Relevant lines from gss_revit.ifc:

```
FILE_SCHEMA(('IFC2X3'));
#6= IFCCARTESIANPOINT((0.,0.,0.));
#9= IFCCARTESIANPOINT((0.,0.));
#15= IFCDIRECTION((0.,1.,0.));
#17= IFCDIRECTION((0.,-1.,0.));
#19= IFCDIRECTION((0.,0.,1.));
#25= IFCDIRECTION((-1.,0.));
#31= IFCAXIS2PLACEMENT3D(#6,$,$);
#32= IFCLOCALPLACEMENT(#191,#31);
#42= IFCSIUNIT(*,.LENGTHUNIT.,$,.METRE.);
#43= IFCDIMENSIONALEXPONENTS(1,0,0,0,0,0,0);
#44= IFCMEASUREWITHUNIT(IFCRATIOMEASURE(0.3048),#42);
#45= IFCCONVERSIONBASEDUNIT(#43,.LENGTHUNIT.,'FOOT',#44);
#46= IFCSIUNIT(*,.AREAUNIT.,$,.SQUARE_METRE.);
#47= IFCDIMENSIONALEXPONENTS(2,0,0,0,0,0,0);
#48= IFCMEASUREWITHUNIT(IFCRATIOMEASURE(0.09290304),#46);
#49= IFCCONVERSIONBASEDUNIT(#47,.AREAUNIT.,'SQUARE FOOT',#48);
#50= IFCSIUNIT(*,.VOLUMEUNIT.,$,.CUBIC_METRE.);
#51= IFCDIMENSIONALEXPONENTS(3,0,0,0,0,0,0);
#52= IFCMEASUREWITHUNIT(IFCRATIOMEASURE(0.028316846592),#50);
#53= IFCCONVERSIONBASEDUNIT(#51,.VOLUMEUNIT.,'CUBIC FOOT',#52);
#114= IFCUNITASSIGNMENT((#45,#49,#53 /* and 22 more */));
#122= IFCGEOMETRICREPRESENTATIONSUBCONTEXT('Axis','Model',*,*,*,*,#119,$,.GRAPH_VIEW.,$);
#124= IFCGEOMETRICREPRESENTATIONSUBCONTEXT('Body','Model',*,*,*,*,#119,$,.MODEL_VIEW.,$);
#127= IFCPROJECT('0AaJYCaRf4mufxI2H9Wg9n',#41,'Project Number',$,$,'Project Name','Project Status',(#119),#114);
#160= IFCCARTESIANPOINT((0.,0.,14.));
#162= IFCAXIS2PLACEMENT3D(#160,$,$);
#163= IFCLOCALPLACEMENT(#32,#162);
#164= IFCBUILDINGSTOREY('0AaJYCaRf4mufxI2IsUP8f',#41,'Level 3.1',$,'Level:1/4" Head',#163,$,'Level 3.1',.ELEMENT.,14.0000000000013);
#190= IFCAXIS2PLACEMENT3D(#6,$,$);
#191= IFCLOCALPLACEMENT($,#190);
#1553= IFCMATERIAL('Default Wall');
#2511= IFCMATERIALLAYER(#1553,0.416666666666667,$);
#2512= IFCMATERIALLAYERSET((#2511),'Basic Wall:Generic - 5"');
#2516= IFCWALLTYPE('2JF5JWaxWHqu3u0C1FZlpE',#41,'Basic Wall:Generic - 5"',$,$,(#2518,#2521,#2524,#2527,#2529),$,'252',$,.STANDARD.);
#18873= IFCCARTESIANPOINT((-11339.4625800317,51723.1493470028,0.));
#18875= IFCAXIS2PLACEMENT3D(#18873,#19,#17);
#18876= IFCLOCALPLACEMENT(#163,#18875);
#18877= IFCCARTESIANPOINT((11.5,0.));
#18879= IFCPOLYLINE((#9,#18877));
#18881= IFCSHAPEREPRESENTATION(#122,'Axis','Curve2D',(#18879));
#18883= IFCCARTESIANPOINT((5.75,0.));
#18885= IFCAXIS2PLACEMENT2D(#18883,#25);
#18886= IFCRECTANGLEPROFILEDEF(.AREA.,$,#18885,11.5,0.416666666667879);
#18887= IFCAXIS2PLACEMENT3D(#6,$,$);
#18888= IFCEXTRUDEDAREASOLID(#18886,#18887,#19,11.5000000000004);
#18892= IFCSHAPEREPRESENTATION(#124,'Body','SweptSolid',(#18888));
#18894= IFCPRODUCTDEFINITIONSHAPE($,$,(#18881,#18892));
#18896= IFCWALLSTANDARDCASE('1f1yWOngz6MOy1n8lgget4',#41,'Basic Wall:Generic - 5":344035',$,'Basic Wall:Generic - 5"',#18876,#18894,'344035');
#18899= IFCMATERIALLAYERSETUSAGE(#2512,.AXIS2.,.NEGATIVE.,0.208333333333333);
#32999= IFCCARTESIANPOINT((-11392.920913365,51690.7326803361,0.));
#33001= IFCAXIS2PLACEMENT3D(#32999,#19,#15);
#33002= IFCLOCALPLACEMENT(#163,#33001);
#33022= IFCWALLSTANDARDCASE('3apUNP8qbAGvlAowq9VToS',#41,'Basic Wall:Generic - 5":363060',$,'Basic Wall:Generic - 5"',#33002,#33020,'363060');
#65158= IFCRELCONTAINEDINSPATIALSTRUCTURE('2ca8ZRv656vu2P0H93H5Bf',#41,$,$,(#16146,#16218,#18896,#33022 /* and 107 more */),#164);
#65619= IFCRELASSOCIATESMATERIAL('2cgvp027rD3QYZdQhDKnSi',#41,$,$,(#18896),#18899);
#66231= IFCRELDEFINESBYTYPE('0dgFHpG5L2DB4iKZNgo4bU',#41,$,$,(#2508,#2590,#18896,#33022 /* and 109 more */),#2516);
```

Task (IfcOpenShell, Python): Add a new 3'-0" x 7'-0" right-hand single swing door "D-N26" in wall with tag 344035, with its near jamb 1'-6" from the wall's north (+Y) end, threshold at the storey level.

```python
import numpy as np
import ifcopenshell
import ifcopenshell.api.feature
import ifcopenshell.api.geometry
import ifcopenshell.api.root
import ifcopenshell.api.spatial
import ifcopenshell.api.type
import ifcopenshell.geom
import ifcopenshell.util.element
import ifcopenshell.util.placement
import ifcopenshell.util.representation
import ifcopenshell.util.shape
import ifcopenshell.util.unit

model = ifcopenshell.open("gss_revit.ifc")
unit_scale = ifcopenshell.util.unit.calculate_unit_scale(model)
settings = ifcopenshell.geom.settings()


def volume(element):
    """Net volume in cubic metres, openings subtracted."""
    shape = ifcopenshell.geom.create_shape(settings, element)
    return ifcopenshell.util.shape.get_volume(shape.geometry)


wall = model.by_guid("1f1yWOngz6MOy1n8lgget4")
storey = ifcopenshell.util.element.get_container(wall, ifc_class="IfcBuildingStorey")
context = ifcopenshell.util.representation.get_context(model, "Model", "Body", "MODEL_VIEW")
before = volume(wall)

width, height, from_end, sill = 0.9144, 2.1336, 0.4572, 0.0  # metres

# The wall runs along its own X axis, and the end named is its -X end.
wall_shape = ifcopenshell.geom.create_shape(settings, wall)
x, y, z = ifcopenshell.util.shape.get_vertices(wall_shape.geometry).T
start = x.min() + from_end
face, thickness = float(y.min()), float(y.max() - y.min())
wall_matrix = ifcopenshell.util.placement.get_local_placement(wall.ObjectPlacement)
level = ifcopenshell.util.placement.get_local_placement(storey.ObjectPlacement)[2, 3]


def in_wall(x, y):
    """Placement at x, y metres in the wall's axes, at sill height."""
    matrix = wall_matrix.copy()
    matrix[:, 3] = wall_matrix @ np.array([x / unit_scale, y / unit_scale, 0.0, 1.0])
    matrix[2, 3] = level + sill / unit_scale
    return matrix


# Opening: a box that overshoots both wall faces by 50 mm.
opening = ifcopenshell.api.root.create_entity(model, ifc_class="IfcOpeningElement")
box = ifcopenshell.api.geometry.add_wall_representation(
    model, context=context, length=width, height=height, thickness=thickness + 0.1
)
ifcopenshell.api.geometry.assign_representation(model, product=opening, representation=box)
ifcopenshell.api.geometry.edit_object_placement(model, product=opening, matrix=in_wall(start, face - 0.05), is_si=False)
ifcopenshell.api.feature.add_feature(model, feature=opening, element=wall)

door = ifcopenshell.api.root.create_entity(model, ifc_class="IfcDoor", name="D-N26")
door.OverallWidth, door.OverallHeight = width / unit_scale, height / unit_scale
body = ifcopenshell.api.geometry.add_door_representation(
    model,
    context=context,
    overall_width=door.OverallWidth,
    overall_height=door.OverallHeight,
    operation_type="SINGLE_SWING_RIGHT",
    lining_properties={"LiningDepth": thickness / unit_scale, "ThresholdDepth": thickness / unit_scale},
)
ifcopenshell.api.geometry.assign_representation(model, product=door, representation=body)
ifcopenshell.api.spatial.assign_container(model, products=[door], relating_structure=storey)
fills = ifcopenshell.api.feature.add_filling(model, opening=opening, element=door)
fills.OwnerHistory = door.OwnerHistory  # required in IFC2X3

# IFC2X3 keeps the operation on the door style.
style = ifcopenshell.api.root.create_entity(model, ifc_class="IfcDoorStyle", name="D-N26")
style.OperationType, style.ConstructionType = "SINGLE_SWING_RIGHT", "NOTDEFINED"
style.ParameterTakesPrecedence = style.Sizeable = False
ifcopenshell.api.type.assign_type(model, related_objects=[door], relating_type=style)

# The lining spans the wall, so the door starts at the wall face.
ifcopenshell.api.geometry.edit_object_placement(model, product=door, matrix=in_wall(start, face), is_si=False)

after = volume(wall)

print(f"wall volume {before:.3f} -> {after:.3f} m3")

model.write("gss_revit_updated.ifc")
```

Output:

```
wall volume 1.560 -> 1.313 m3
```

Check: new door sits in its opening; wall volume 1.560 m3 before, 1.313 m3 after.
